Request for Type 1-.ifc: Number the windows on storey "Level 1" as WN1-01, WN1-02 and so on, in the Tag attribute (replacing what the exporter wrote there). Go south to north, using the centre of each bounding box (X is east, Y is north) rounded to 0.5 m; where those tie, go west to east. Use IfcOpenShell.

First a look at what the model holds.

```python
import ifcopenshell
import ifcopenshell.util.element
import ifcopenshell.util.placement

model = ifcopenshell.open("Type 1-.ifc")
print(model.schema)
storey = next(s for s in model.by_type("IfcBuildingStorey") if s.Name == "Level 1")
windows = [e for e in ifcopenshell.util.element.get_decomposition(storey) if e.is_a("IfcWindow")]
for e in sorted(windows, key=lambda e: e.id()):
    origin = ifcopenshell.util.placement.get_local_placement(e.ObjectPlacement)[:3, 3]
    print(e.id(), e.Tag, e.Name, origin.round(2) + 0.0, sep=" | ")
```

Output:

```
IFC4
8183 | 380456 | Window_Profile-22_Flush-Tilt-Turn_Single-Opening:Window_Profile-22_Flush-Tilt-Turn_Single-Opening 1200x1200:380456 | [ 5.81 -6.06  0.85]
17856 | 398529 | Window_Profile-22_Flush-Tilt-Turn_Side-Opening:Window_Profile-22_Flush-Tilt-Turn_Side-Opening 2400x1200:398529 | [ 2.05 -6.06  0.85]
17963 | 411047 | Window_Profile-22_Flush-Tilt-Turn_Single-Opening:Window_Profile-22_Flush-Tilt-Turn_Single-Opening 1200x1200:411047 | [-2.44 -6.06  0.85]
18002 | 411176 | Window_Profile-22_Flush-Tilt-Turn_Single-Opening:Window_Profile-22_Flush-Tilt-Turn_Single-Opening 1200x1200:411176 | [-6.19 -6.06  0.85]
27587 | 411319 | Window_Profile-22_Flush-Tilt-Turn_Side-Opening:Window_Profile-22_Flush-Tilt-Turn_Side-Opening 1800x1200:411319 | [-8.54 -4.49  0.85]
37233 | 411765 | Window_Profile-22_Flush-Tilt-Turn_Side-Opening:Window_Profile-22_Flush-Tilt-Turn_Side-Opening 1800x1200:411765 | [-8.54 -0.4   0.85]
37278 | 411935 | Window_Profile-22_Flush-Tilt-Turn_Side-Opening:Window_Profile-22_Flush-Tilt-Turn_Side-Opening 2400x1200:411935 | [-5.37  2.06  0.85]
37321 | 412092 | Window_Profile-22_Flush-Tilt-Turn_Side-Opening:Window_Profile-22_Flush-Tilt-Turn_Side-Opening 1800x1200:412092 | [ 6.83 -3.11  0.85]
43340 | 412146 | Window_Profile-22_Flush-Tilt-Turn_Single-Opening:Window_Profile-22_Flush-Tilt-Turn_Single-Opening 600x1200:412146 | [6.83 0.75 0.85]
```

```python
import ifcopenshell
import ifcopenshell.geom
import ifcopenshell.util.element
import ifcopenshell.util.shape

model = ifcopenshell.open("Type 1-.ifc")
settings = ifcopenshell.geom.settings()
settings.set("use-world-coords", True)


def centre(element):
    shape = ifcopenshell.geom.create_shape(settings, element)
    return ifcopenshell.util.shape.get_bbox_centroid(shape.geometry)


storey = next(s for s in model.by_type("IfcBuildingStorey") if s.Name == "Level 1")
windows = [e for e in ifcopenshell.util.element.get_decomposition(storey) if e.is_a("IfcWindow")]

# Insertion points can sit at a corner or the storey origin, so sort by the geometry (in metres).
centres = {e: centre(e) for e in windows}
windows.sort(key=lambda e: (round(centres[e][1] / 0.5), centres[e][0]))

for i, e in enumerate(windows, start=1):
    number = f"WN1-{i:02d}"
    e.Tag = number
    print(e.id(), number)

model.write("Type 1-_rev.ifc")
```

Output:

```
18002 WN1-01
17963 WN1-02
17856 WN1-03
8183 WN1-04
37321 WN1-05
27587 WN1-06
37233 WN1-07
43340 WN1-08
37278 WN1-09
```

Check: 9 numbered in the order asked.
